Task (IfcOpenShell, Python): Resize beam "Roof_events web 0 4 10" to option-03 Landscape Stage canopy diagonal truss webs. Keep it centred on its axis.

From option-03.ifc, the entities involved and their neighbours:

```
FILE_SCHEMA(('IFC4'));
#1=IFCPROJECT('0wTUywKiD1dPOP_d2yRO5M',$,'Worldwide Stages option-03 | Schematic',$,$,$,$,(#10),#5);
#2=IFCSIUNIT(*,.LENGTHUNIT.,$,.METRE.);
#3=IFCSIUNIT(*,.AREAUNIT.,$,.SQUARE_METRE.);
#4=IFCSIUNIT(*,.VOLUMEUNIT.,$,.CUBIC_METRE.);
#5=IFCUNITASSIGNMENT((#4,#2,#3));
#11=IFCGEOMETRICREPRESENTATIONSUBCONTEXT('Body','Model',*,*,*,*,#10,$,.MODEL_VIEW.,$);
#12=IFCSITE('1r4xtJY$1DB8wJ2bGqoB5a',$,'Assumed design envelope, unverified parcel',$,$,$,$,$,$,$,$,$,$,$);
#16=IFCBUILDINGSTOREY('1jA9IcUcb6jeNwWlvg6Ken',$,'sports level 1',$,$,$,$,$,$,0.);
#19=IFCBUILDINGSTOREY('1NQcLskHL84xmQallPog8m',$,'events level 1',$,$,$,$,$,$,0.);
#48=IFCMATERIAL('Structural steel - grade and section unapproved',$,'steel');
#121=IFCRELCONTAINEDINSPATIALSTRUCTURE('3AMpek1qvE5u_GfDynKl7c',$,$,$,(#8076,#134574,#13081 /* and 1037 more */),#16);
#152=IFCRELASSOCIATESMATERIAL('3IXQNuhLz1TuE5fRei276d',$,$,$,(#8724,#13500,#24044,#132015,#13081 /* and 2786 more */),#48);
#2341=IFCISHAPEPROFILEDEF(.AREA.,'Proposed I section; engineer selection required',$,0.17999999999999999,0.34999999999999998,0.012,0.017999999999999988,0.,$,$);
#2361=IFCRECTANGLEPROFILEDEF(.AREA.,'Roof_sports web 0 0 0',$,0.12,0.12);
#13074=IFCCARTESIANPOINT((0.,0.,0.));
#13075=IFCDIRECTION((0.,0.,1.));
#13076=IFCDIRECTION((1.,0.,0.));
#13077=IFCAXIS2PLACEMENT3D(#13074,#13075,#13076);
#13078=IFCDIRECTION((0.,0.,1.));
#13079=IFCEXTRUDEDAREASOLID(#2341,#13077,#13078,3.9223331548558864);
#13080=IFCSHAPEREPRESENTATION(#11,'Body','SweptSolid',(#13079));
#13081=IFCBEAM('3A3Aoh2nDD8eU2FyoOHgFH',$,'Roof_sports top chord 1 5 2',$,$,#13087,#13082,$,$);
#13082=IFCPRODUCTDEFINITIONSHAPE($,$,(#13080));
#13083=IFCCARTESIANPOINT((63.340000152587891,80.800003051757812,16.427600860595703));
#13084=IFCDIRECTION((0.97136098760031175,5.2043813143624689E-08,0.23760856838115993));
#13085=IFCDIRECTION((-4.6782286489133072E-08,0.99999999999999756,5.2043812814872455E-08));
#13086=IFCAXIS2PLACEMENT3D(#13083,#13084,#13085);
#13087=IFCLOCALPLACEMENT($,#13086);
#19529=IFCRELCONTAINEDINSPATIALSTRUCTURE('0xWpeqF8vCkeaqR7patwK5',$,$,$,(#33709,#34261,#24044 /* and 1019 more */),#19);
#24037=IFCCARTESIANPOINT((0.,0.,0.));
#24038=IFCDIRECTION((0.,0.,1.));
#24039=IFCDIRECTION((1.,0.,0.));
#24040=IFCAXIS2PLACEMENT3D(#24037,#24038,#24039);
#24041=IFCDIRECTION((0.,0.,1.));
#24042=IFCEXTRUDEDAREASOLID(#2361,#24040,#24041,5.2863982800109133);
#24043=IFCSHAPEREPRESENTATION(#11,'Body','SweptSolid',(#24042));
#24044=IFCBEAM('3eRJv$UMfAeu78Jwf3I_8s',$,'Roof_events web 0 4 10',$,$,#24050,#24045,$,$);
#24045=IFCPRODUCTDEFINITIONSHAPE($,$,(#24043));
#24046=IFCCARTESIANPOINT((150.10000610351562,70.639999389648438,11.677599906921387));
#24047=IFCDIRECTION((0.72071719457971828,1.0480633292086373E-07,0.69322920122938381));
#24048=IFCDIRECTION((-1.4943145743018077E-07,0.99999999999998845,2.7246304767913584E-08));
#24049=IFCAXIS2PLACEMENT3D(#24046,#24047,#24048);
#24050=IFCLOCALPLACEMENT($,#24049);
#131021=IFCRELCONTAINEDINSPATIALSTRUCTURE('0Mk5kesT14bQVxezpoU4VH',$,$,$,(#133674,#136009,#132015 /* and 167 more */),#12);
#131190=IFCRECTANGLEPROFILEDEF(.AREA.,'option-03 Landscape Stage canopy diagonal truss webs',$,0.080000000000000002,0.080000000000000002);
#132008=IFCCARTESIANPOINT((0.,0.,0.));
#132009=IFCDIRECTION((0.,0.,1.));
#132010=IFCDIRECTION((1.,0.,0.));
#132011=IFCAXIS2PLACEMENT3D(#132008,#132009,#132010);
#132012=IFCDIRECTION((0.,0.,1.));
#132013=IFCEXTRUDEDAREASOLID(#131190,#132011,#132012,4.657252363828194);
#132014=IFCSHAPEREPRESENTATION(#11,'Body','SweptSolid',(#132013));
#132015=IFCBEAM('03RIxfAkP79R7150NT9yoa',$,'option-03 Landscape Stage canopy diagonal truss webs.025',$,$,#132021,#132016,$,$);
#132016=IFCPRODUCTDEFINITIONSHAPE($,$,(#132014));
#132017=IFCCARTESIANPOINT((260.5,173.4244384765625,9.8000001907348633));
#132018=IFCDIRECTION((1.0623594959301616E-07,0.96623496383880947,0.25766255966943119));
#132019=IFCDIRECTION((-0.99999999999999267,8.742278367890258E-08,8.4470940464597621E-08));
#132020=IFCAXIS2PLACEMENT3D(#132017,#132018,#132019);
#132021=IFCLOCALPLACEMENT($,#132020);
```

```python
import ifcopenshell
import ifcopenshell.util.element
import ifcopenshell.util.representation

model = ifcopenshell.open("option-03.ifc")

member = model.by_guid("3eRJv$UMfAeu78Jwf3I_8s")
source = next(p for p in model.by_type("IfcRectangleProfileDef") if p.ProfileName == "option-03 Landscape Stage canopy diagonal truss webs")

body = ifcopenshell.util.representation.get_representation(member, "Model", "Body")
solid = body.Items[0]
old_profile = solid.SweptArea

# Copy the section's sizes but keep this member's own profile position.
profile = ifcopenshell.util.element.copy(model, source)
profile.Position = old_profile.Position
solid.SweptArea = profile
if not model.get_total_inverses(old_profile):
    ifcopenshell.util.element.remove_deep2(model, old_profile)

print(solid.SweptArea)

model.write("option-03_rev.ifc")
```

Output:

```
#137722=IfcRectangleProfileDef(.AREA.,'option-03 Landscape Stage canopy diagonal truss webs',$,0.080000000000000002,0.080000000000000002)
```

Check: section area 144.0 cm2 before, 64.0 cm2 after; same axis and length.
